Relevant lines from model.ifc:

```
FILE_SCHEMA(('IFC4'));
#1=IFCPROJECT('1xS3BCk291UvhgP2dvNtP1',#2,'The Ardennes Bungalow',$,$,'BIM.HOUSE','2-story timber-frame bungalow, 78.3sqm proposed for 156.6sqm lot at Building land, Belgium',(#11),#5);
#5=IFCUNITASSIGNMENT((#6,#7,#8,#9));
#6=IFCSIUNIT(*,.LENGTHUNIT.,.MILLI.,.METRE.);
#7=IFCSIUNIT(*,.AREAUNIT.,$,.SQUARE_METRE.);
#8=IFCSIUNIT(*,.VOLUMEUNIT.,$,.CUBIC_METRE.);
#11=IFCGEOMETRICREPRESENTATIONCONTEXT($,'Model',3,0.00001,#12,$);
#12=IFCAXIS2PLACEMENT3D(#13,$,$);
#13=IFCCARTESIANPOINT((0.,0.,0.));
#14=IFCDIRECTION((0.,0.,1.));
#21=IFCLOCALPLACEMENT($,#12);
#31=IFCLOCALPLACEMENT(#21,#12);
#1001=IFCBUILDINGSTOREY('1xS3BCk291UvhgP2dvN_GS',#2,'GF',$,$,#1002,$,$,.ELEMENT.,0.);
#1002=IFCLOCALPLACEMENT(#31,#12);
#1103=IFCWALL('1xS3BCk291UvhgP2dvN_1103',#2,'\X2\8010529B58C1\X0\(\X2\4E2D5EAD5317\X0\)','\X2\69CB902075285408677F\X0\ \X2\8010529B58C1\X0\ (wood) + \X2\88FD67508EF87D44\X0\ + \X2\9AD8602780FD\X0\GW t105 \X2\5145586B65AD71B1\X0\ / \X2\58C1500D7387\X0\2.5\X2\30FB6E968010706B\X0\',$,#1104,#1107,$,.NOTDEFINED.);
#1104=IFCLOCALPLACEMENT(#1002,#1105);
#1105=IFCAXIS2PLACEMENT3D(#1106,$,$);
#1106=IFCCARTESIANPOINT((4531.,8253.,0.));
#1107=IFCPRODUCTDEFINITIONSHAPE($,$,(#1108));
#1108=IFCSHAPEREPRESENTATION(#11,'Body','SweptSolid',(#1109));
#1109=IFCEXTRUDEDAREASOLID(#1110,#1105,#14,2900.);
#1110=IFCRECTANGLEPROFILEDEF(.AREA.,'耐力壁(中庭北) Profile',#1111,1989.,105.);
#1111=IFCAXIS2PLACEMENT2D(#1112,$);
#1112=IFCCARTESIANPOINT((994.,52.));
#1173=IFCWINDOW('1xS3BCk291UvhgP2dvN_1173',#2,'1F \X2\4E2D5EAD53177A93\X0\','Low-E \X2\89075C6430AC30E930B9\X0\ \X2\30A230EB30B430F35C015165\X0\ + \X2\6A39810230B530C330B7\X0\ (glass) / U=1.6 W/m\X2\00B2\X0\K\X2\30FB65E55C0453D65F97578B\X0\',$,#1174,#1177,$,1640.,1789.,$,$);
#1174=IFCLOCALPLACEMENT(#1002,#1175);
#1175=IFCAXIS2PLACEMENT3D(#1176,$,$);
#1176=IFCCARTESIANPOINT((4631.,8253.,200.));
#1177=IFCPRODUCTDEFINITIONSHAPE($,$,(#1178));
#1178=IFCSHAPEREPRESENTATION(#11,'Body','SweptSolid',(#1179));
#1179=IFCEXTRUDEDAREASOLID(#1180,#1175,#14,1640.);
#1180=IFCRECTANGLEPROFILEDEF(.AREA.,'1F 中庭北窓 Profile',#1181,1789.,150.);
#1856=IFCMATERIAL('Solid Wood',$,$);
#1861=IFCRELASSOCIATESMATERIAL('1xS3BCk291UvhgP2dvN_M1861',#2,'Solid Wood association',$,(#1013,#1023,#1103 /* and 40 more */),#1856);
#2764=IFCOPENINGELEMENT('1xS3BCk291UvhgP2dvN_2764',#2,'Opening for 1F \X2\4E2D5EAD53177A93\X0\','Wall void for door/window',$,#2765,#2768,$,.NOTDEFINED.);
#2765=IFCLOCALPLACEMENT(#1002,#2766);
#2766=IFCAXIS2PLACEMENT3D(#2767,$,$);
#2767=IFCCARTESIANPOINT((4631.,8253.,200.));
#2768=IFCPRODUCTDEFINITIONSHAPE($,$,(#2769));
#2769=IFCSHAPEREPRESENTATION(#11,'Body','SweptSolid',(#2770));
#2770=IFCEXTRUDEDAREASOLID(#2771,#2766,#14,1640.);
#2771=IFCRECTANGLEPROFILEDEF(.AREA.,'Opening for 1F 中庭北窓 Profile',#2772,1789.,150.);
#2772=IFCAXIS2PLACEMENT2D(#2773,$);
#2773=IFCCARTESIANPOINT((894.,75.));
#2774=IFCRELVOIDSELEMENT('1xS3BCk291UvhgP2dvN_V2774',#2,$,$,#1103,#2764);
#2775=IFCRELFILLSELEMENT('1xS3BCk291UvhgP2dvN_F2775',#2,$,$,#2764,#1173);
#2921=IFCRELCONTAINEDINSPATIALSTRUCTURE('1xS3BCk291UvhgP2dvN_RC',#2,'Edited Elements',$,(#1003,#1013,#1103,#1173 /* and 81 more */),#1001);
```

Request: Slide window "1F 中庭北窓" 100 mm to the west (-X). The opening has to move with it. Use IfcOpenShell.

```python
import ifcopenshell
import ifcopenshell.api.geometry
import ifcopenshell.util.placement
import ifcopenshell.util.unit

model = ifcopenshell.open("model.ifc")
unit_scale = ifcopenshell.util.unit.calculate_unit_scale(model)

window = model.by_guid("1xS3BCk291UvhgP2dvN_1173")
opening = window.FillsVoids[0].RelatingOpeningElement
wall = opening.VoidsElements[0].RelatingBuildingElement

wall_matrix = ifcopenshell.util.placement.get_local_placement(wall.ObjectPlacement)
shift = wall_matrix[:3, 0] * -0.1 / unit_scale
before = ifcopenshell.util.placement.get_local_placement(window.ObjectPlacement)[:3, 3].copy()

# The window is not placed relative to its opening, so move both.
for product in (opening, window):
    matrix = ifcopenshell.util.placement.get_local_placement(product.ObjectPlacement)
    matrix[:3, 3] += shift
    ifcopenshell.api.geometry.edit_object_placement(model, product=product, matrix=matrix, is_si=False)

after = ifcopenshell.util.placement.get_local_placement(window.ObjectPlacement)[:3, 3]
print("window moved by", (after - before).round(3) + 0.0)

model.write("model_updated.ifc")
```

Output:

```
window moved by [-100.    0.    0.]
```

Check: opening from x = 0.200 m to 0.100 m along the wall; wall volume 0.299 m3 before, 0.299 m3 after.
